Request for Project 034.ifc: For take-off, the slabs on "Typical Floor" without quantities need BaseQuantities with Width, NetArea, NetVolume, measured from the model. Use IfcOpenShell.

First a look at what the model holds.

```python
import ifcopenshell
import ifcopenshell.util.element
import ifcopenshell.util.unit

model = ifcopenshell.open("Project 034.ifc")
print(model.schema)
for unit_type in ("LENGTHUNIT", "AREAUNIT", "VOLUMEUNIT"):
    print(unit_type, ifcopenshell.util.unit.calculate_unit_scale(model, unit_type))
storey = next(s for s in model.by_type("IfcBuildingStorey") if s.Name == "Typical Floor")
slabs = [e for e in ifcopenshell.util.element.get_decomposition(storey) if e.is_a("IfcSlab")]
for e in sorted(slabs, key=lambda e: e.id()):
    print(e.id(), e.is_a(), e.Name, list(ifcopenshell.util.element.get_psets(e, qtos_only=True)), sep=" | ")
```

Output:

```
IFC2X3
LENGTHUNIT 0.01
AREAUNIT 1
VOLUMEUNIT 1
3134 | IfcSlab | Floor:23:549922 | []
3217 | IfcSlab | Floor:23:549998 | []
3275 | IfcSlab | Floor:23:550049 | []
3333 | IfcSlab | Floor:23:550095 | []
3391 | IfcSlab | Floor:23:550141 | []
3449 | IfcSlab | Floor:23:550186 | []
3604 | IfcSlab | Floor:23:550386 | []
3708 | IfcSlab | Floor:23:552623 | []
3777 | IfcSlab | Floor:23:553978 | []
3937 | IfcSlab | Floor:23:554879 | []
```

```python
import ifcopenshell
import ifcopenshell.api.pset
import ifcopenshell.geom
import ifcopenshell.util.element
import ifcopenshell.util.shape
import ifcopenshell.util.unit

model = ifcopenshell.open("Project 034.ifc")
unit_scale = ifcopenshell.util.unit.calculate_unit_scale(model)
area_scale = ifcopenshell.util.unit.calculate_unit_scale(model, "AREAUNIT")
volume_scale = ifcopenshell.util.unit.calculate_unit_scale(model, "VOLUMEUNIT")
settings = ifcopenshell.geom.settings()

storey = next(s for s in model.by_type("IfcBuildingStorey") if s.Name == "Typical Floor")
slabs = [e for e in ifcopenshell.util.element.get_decomposition(storey) if e.is_a("IfcSlab")]

for e in sorted(slabs, key=lambda e: e.id()):
    if ifcopenshell.util.element.get_psets(e, qtos_only=True, should_inherit=False):
        continue
    # Geometry comes back in metres, in the element's own axes.
    shape = ifcopenshell.geom.create_shape(settings, e)
    values = {
        "Width": ifcopenshell.util.shape.get_z(shape.geometry) / unit_scale,
        "NetArea": ifcopenshell.util.shape.get_footprint_area(shape.geometry) / area_scale,
        "NetVolume": ifcopenshell.util.shape.get_volume(shape.geometry) / volume_scale,
    }
    qto = ifcopenshell.api.pset.add_qto(model, product=e, name="BaseQuantities")
    ifcopenshell.api.pset.edit_qto(model, qto=qto, properties=values)
    print(e.id(), {k: round(v, 3) for k, v in values.items()})

model.write("Project 034_rev.ifc")
```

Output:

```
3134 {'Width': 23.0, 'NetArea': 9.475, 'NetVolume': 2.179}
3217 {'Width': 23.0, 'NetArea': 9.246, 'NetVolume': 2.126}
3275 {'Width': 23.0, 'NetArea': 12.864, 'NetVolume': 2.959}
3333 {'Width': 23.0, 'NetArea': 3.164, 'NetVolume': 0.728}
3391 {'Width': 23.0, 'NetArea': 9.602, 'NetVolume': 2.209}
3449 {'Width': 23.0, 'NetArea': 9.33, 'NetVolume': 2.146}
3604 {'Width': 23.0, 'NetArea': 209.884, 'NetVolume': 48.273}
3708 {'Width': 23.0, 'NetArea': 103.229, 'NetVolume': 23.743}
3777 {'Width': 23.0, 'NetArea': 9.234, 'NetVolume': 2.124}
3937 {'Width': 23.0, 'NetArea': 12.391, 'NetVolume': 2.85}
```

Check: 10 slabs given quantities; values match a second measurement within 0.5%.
